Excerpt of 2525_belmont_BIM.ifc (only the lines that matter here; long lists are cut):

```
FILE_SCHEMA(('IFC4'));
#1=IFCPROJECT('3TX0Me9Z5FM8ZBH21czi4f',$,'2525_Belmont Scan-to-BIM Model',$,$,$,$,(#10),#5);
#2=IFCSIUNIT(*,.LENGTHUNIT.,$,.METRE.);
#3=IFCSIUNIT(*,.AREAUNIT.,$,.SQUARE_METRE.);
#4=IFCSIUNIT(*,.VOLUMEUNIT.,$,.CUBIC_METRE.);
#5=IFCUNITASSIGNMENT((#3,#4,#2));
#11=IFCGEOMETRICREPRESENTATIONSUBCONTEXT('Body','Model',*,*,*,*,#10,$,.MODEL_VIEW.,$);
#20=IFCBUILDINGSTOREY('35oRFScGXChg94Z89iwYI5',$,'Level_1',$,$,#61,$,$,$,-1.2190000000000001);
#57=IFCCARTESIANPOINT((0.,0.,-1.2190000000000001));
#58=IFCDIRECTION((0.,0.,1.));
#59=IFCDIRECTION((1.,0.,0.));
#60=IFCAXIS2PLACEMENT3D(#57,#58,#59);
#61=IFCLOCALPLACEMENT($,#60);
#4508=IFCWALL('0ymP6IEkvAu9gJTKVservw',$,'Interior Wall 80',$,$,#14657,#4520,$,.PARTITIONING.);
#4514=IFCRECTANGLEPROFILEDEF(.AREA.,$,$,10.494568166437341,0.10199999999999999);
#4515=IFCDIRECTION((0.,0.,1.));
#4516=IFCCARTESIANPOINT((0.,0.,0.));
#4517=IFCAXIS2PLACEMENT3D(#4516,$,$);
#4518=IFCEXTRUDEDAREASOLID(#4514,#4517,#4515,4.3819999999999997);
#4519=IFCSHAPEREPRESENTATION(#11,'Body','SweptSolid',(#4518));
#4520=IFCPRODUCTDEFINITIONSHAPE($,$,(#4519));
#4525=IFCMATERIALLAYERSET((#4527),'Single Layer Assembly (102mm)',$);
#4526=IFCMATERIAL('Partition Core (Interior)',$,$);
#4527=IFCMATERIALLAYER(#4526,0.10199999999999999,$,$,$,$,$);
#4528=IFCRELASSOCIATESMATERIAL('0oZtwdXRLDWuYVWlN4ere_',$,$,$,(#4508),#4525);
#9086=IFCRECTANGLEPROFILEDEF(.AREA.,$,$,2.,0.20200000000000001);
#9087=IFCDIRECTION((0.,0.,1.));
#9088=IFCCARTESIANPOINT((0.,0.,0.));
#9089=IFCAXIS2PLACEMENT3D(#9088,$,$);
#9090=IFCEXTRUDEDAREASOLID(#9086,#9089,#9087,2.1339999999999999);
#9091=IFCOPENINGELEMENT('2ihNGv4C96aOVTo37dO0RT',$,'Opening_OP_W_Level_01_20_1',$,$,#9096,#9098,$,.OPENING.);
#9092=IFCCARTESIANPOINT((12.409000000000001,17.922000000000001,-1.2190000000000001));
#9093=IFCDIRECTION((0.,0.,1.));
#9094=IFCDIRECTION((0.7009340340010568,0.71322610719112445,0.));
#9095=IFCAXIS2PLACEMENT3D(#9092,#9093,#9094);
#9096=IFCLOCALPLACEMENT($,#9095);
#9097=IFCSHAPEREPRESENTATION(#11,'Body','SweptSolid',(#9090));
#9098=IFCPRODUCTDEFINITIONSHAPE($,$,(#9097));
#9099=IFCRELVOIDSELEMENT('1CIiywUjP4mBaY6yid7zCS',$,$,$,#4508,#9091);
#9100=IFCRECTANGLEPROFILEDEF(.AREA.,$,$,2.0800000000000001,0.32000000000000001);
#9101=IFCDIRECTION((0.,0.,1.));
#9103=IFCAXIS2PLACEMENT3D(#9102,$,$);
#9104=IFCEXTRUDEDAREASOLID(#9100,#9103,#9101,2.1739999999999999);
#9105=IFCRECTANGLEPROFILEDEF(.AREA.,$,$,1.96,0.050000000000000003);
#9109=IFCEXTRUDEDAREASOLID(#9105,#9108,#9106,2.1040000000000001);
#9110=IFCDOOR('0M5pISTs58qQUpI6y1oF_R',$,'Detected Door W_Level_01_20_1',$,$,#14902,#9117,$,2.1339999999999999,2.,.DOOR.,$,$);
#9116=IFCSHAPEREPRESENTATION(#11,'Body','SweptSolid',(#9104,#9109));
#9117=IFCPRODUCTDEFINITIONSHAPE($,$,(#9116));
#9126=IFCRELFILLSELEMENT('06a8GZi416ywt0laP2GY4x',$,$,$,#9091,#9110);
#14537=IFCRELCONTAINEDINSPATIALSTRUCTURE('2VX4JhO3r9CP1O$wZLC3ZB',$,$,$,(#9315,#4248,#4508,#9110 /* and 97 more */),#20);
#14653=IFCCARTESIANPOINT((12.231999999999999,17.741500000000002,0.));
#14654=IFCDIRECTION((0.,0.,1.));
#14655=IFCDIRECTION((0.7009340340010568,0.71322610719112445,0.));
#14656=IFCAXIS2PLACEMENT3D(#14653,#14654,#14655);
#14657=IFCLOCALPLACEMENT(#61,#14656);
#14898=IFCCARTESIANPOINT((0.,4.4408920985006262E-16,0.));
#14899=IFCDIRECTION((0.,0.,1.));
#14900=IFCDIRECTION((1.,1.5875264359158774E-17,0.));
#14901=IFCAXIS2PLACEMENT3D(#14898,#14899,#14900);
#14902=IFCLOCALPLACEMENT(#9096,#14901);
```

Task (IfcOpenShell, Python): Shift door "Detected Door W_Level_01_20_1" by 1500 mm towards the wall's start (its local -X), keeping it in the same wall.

```python
import ifcopenshell
import ifcopenshell.api.geometry
import ifcopenshell.util.placement

model = ifcopenshell.open("2525_belmont_BIM.ifc")

door = model.by_guid("0M5pISTs58qQUpI6y1oF_R")
opening = door.FillsVoids[0].RelatingOpeningElement
wall = opening.VoidsElements[0].RelatingBuildingElement

wall_matrix = ifcopenshell.util.placement.get_local_placement(wall.ObjectPlacement)
shift = wall_matrix[:3, 0] * -1.5
before = ifcopenshell.util.placement.get_local_placement(door.ObjectPlacement)[:3, 3].copy()

# The door is placed relative to its opening, so it follows when the opening moves.
matrix = ifcopenshell.util.placement.get_local_placement(opening.ObjectPlacement)
matrix[:3, 3] += shift
ifcopenshell.api.geometry.edit_object_placement(
    model, product=opening, matrix=matrix, is_si=False, should_transform_children=True
)

after = ifcopenshell.util.placement.get_local_placement(door.ObjectPlacement)[:3, 3]
print("door moved by", (after - before).round(3) + 0.0)

model.write("2525_belmont_BIM_edited.ifc")
```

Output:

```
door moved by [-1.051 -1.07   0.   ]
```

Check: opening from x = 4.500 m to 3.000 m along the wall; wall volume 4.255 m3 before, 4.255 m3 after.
